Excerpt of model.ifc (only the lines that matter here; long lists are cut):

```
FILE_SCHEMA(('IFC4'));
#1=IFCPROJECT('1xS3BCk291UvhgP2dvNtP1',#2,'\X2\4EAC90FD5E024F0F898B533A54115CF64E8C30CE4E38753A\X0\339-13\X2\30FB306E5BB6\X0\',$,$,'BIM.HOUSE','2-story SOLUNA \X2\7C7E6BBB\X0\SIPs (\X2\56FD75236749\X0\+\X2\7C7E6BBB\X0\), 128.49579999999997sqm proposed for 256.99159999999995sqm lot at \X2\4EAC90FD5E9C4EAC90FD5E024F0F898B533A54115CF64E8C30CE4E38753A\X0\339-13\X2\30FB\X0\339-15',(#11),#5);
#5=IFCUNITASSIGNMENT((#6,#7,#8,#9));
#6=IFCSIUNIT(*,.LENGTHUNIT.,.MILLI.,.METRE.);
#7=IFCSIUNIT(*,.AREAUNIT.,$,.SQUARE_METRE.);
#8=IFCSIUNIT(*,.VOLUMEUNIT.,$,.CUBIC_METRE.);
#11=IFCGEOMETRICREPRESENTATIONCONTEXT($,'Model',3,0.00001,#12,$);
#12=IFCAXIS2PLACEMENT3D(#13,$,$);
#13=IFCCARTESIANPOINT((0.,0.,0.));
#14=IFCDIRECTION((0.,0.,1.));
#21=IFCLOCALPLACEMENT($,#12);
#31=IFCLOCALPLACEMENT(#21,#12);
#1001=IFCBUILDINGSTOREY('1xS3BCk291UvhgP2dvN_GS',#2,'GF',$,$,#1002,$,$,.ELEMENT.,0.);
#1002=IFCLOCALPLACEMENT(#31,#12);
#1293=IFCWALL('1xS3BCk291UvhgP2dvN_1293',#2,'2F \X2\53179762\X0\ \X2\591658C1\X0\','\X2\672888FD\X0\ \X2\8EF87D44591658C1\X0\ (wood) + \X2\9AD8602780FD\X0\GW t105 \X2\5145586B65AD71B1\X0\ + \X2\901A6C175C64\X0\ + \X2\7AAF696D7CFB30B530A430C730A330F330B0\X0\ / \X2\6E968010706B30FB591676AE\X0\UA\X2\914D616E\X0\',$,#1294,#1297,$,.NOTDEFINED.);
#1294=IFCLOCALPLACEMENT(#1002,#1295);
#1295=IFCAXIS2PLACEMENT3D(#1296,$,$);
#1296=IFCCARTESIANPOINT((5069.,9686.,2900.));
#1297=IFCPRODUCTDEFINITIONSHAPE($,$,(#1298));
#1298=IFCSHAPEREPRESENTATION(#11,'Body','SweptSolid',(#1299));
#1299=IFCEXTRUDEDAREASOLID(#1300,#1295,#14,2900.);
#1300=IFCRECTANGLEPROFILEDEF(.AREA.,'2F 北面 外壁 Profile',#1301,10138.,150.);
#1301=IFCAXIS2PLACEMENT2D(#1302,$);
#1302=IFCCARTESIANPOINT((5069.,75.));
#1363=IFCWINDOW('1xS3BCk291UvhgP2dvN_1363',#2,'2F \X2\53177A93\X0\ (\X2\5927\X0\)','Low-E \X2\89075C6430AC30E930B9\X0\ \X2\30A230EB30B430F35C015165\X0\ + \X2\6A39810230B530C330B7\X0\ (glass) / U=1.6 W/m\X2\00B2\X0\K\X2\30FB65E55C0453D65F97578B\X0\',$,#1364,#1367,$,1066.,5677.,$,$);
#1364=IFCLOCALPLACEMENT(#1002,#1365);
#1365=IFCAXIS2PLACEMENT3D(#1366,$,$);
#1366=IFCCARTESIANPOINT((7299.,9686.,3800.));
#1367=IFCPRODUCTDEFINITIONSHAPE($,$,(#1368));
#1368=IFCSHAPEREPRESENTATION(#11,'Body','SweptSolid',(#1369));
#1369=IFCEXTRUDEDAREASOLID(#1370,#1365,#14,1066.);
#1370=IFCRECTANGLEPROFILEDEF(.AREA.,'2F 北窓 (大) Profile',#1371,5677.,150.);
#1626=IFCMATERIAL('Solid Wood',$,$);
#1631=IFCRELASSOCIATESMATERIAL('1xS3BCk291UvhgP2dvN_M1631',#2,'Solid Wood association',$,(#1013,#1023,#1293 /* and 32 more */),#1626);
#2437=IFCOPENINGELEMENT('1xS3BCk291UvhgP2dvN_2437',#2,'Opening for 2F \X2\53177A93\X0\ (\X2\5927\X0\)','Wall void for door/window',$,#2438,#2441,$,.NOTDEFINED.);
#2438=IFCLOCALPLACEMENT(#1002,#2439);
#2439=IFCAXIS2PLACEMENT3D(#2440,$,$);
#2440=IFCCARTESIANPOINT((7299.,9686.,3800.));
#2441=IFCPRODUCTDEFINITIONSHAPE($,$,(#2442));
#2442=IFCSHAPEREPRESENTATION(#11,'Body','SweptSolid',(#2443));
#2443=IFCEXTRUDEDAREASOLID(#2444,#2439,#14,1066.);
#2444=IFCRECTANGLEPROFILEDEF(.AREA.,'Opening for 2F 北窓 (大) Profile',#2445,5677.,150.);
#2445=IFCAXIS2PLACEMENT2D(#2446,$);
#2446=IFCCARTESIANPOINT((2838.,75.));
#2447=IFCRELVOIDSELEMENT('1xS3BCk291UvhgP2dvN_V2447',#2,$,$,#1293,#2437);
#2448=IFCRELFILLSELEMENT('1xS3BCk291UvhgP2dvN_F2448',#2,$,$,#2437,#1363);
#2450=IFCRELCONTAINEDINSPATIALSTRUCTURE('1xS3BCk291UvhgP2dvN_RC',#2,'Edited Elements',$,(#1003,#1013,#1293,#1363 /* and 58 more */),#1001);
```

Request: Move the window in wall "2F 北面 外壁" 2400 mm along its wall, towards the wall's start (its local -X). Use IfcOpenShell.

```python
import ifcopenshell
import ifcopenshell.api.geometry
import ifcopenshell.util.placement

model = ifcopenshell.open("model.ifc")

window = model.by_guid("1xS3BCk291UvhgP2dvN_1363")
opening = window.FillsVoids[0].RelatingOpeningElement
wall = opening.VoidsElements[0].RelatingBuildingElement

wall_matrix = ifcopenshell.util.placement.get_local_placement(wall.ObjectPlacement)
shift = wall_matrix[:3, 0] * -2400.0
before = ifcopenshell.util.placement.get_local_placement(window.ObjectPlacement)[:3, 3].copy()

# The window is not placed relative to its opening, so move both.
for product in (opening, window):
    matrix = ifcopenshell.util.placement.get_local_placement(product.ObjectPlacement)
    matrix[:3, 3] += shift
    ifcopenshell.api.geometry.edit_object_placement(model, product=product, matrix=matrix, is_si=False)

after = ifcopenshell.util.placement.get_local_placement(window.ObjectPlacement)[:3, 3]
print("window moved by", (after - before).round(3) + 0.0)

model.write("model_v2.ifc")
```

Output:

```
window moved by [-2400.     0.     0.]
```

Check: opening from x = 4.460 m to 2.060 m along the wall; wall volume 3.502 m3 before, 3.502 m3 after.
